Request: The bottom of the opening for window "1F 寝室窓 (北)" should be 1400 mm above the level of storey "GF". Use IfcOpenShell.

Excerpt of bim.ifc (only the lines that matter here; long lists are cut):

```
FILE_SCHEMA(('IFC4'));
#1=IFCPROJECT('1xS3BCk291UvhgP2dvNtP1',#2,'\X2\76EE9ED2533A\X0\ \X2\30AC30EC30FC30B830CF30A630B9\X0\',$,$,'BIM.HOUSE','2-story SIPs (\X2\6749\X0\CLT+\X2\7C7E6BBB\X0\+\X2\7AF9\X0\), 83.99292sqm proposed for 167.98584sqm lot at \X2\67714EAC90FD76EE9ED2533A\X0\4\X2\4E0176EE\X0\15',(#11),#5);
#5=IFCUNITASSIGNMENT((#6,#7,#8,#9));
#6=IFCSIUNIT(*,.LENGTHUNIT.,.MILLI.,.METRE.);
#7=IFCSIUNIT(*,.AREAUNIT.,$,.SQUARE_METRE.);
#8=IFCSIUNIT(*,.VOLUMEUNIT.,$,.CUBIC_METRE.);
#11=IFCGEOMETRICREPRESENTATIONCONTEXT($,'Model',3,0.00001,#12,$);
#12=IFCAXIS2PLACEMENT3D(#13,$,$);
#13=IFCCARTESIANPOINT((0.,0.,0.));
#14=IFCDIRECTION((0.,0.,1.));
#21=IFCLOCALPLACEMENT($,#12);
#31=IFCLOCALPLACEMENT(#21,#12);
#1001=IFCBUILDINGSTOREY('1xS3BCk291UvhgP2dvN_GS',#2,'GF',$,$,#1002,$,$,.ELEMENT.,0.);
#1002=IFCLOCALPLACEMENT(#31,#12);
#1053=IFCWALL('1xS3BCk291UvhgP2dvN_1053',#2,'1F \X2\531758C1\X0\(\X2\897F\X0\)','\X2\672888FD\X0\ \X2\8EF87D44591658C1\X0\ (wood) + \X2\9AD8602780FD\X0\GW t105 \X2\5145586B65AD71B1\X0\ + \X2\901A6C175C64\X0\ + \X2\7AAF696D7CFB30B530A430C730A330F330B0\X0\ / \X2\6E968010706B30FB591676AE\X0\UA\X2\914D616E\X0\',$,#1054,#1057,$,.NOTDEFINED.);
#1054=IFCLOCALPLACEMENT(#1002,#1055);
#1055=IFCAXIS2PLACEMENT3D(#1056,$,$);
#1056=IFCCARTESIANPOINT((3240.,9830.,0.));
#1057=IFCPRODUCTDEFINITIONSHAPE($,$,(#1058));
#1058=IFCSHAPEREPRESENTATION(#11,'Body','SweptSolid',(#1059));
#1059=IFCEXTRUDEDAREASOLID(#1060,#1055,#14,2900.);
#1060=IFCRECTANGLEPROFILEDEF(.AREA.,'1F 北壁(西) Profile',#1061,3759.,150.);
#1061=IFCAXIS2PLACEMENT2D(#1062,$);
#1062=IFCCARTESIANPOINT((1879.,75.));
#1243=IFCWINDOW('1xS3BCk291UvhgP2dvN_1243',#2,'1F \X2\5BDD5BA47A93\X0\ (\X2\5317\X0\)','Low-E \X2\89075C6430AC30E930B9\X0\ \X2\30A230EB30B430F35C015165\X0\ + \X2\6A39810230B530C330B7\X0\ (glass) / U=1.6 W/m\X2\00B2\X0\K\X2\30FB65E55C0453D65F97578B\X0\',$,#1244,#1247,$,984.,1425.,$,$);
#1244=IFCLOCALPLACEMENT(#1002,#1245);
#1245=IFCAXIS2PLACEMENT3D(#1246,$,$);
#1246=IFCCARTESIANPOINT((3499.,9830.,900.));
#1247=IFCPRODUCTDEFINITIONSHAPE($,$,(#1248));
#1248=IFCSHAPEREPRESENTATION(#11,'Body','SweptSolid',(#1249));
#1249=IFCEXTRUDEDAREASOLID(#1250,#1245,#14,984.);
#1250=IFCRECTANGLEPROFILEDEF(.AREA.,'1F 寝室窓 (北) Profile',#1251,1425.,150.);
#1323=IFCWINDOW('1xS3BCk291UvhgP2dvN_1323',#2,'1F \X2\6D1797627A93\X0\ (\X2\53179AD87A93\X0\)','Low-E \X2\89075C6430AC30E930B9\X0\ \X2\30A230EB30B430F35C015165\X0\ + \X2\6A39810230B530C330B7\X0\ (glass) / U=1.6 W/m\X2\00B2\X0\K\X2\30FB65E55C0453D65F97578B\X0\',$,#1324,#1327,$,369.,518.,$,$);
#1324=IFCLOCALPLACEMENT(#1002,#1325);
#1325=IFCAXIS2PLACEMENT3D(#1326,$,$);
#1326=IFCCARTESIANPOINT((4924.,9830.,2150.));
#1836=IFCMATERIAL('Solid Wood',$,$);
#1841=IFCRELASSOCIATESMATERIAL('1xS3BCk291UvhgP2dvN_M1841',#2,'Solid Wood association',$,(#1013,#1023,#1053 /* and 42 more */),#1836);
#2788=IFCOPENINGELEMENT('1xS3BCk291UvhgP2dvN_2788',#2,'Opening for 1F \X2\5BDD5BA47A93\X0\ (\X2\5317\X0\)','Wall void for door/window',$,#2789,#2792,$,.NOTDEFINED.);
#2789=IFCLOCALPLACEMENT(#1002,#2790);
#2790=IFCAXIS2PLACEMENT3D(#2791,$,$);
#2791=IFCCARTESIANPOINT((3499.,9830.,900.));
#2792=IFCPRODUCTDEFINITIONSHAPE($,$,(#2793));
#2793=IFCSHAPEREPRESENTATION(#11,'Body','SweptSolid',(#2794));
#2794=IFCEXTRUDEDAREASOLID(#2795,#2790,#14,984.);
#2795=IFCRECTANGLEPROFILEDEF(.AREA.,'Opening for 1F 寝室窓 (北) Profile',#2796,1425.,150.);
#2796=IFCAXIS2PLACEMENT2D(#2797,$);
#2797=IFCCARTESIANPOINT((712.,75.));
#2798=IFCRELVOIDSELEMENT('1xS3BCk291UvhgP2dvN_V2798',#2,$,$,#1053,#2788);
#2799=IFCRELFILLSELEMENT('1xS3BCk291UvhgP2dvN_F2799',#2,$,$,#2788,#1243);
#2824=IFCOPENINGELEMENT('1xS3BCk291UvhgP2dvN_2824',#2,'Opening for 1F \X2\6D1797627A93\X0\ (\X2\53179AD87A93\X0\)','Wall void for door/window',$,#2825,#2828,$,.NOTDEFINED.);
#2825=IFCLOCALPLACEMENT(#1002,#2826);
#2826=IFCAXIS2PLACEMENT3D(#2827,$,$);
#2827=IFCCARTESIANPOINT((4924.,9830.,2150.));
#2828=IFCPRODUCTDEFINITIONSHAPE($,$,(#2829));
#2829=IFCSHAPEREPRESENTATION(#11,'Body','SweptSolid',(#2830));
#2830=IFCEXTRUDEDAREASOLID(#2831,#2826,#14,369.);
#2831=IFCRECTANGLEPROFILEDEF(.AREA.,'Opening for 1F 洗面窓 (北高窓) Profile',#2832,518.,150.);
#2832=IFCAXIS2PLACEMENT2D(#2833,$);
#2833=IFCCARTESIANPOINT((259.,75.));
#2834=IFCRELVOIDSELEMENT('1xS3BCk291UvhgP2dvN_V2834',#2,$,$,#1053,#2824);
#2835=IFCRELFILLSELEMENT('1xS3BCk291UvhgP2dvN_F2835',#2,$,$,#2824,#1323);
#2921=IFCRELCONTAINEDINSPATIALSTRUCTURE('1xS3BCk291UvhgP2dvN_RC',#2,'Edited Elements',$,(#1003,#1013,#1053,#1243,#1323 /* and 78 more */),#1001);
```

```python
import numpy as np
import ifcopenshell
import ifcopenshell.api.geometry
import ifcopenshell.geom
import ifcopenshell.util.element
import ifcopenshell.util.placement
import ifcopenshell.util.shape
import ifcopenshell.util.unit

model = ifcopenshell.open("bim.ifc")
unit_scale = ifcopenshell.util.unit.calculate_unit_scale(model)

window = model.by_guid("1xS3BCk291UvhgP2dvN_1243")
opening = window.FillsVoids[0].RelatingOpeningElement
storey = ifcopenshell.util.element.get_container(window, ifc_class="IfcBuildingStorey")
level = ifcopenshell.util.placement.get_local_placement(storey.ObjectPlacement)[2, 3]

# The opening's origin need not be at the sill, so measure its lowest point.
shape = ifcopenshell.geom.create_shape(ifcopenshell.geom.settings(), opening)
bottom = ifcopenshell.util.shape.get_shape_bottom_elevation(shape, shape.geometry) / unit_scale
dz = level + 1400.0 - bottom

shift = np.array([0.0, 0.0, dz])
# The window is not placed relative to its opening, so move both.
for product in (opening, window):
    matrix = ifcopenshell.util.placement.get_local_placement(product.ObjectPlacement)
    matrix[:3, 3] += shift
    ifcopenshell.api.geometry.edit_object_placement(model, product=product, matrix=matrix, is_si=False)

print(f"moved by {dz * unit_scale:+.3f} m")

model.write("bim_updated.ifc")
```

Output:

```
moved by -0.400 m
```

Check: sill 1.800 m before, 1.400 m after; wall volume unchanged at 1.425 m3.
